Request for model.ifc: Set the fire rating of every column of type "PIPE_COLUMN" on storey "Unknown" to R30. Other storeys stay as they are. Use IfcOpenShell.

First a look at what the model holds.

```python
import ifcopenshell
import ifcopenshell.util.element

model = ifcopenshell.open("model.ifc")
print(model.schema)
storey = next(s for s in model.by_type("IfcBuildingStorey") if s.Name == "Unknown")
columns = [e for e in ifcopenshell.util.element.get_decomposition(storey) if e.is_a("IfcColumn")]
seen = {}
for e in columns:
    element_type = ifcopenshell.util.element.get_type(e)
    key = (element_type.Name if element_type != e and element_type else None, ifcopenshell.util.element.get_pset(e, "Pset_ColumnCommon", "FireRating"))
    seen[key] = seen.get(key, 0) + 1
for (name, value), count in sorted(seen.items(), key=str):
    print(count, "x", name, "|", value)
```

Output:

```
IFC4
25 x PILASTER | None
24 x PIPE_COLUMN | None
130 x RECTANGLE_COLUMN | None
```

```python
import ifcopenshell
import ifcopenshell.api.pset
import ifcopenshell.util.element

model = ifcopenshell.open("model.ifc")

storey = next(s for s in model.by_type("IfcBuildingStorey") if s.Name == "Unknown")
columns = [e for e in ifcopenshell.util.element.get_decomposition(storey) if e.is_a("IfcColumn")]

count = 0
for e in columns:
    element_type = ifcopenshell.util.element.get_type(e)
    if element_type in (None, e) or element_type.Name != "PIPE_COLUMN":
        continue
    found = ifcopenshell.util.element.get_pset(e, "Pset_ColumnCommon", should_inherit=False)
    if found:
        pset = model.by_id(found["id"])
        if len(ifcopenshell.util.element.get_elements_by_pset(pset)) > 1:
            pset = ifcopenshell.api.pset.unshare_pset(model, products=[e], pset=pset)[0]
    else:
        pset = ifcopenshell.api.pset.add_pset(model, product=e, name="Pset_ColumnCommon")
    ifcopenshell.api.pset.edit_pset(model, pset=pset, properties={"FireRating": "R30"})
    count += 1

print(count, "columns updated")

model.write("model-out.ifc")
```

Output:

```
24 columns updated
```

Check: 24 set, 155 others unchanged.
